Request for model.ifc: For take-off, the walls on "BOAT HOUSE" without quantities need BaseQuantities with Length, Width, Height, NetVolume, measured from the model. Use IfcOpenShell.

First a look at what the model holds.

```python
import ifcopenshell
import ifcopenshell.util.element
import ifcopenshell.util.unit

model = ifcopenshell.open("model.ifc")
print(model.schema)
for unit_type in ("LENGTHUNIT", "AREAUNIT", "VOLUMEUNIT"):
    print(unit_type, ifcopenshell.util.unit.calculate_unit_scale(model, unit_type))
storey = next(s for s in model.by_type("IfcBuildingStorey") if s.Name == "BOAT HOUSE")
walls = [e for e in ifcopenshell.util.element.get_decomposition(storey) if e.is_a("IfcWall")]
for e in sorted(walls, key=lambda e: e.id()):
    print(e.id(), e.is_a(), e.Name, list(ifcopenshell.util.element.get_psets(e, qtos_only=True)), sep=" | ")
```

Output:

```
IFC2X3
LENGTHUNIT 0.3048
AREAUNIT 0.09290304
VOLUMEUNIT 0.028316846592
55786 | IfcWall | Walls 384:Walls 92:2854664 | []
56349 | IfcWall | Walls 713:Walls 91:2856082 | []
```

```python
import ifcopenshell
import ifcopenshell.api.pset
import ifcopenshell.geom
import ifcopenshell.util.element
import ifcopenshell.util.shape
import ifcopenshell.util.unit

model = ifcopenshell.open("model.ifc")
unit_scale = ifcopenshell.util.unit.calculate_unit_scale(model)
volume_scale = ifcopenshell.util.unit.calculate_unit_scale(model, "VOLUMEUNIT")
settings = ifcopenshell.geom.settings()

storey = next(s for s in model.by_type("IfcBuildingStorey") if s.Name == "BOAT HOUSE")
walls = [e for e in ifcopenshell.util.element.get_decomposition(storey) if e.is_a("IfcWall")]

for e in sorted(walls, key=lambda e: e.id()):
    if ifcopenshell.util.element.get_psets(e, qtos_only=True, should_inherit=False):
        continue
    # Geometry comes back in metres, in the element's own axes.
    shape = ifcopenshell.geom.create_shape(settings, e)
    values = {
        "Length": ifcopenshell.util.shape.get_x(shape.geometry) / unit_scale,
        "Width": ifcopenshell.util.shape.get_y(shape.geometry) / unit_scale,
        "Height": ifcopenshell.util.shape.get_z(shape.geometry) / unit_scale,
        "NetVolume": ifcopenshell.util.shape.get_volume(shape.geometry) / volume_scale,
    }
    qto = ifcopenshell.api.pset.add_qto(model, product=e, name="BaseQuantities")
    ifcopenshell.api.pset.edit_qto(model, qto=qto, properties=values)
    print(e.id(), {k: round(v, 3) for k, v in values.items()})

model.write("model_edited.ifc")
```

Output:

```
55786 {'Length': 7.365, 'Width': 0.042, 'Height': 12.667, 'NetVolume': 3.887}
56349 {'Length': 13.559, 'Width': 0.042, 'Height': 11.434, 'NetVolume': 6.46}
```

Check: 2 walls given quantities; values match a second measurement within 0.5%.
